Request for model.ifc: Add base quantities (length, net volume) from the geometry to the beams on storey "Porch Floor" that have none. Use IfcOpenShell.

First a look at what the model holds.

```python
import ifcopenshell
import ifcopenshell.util.element
import ifcopenshell.util.unit

model = ifcopenshell.open("model.ifc")
print(model.schema)
for unit_type in ("LENGTHUNIT", "AREAUNIT", "VOLUMEUNIT"):
    print(unit_type, ifcopenshell.util.unit.calculate_unit_scale(model, unit_type))
storey = next(s for s in model.by_type("IfcBuildingStorey") if s.Name == "Porch Floor")
beams = [e for e in ifcopenshell.util.element.get_decomposition(storey) if e.is_a("IfcBeam")]
for e in sorted(beams, key=lambda e: e.id()):
    print(e.id(), e.is_a(), e.Name, list(ifcopenshell.util.element.get_psets(e, qtos_only=True)), sep=" | ")
```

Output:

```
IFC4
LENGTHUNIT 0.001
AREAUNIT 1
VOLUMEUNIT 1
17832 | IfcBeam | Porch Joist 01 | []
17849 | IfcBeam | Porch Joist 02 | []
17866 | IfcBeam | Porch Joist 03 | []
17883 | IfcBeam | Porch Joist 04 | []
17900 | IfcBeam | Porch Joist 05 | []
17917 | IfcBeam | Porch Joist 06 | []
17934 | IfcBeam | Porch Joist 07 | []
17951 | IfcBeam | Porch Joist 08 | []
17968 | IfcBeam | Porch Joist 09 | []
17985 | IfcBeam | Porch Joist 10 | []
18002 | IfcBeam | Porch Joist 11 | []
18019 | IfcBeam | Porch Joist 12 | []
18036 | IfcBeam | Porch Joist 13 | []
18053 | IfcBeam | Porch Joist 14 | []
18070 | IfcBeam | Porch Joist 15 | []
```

```python
import ifcopenshell
import ifcopenshell.api.pset
import ifcopenshell.geom
import ifcopenshell.util.element
import ifcopenshell.util.shape
import ifcopenshell.util.unit

model = ifcopenshell.open("model.ifc")
unit_scale = ifcopenshell.util.unit.calculate_unit_scale(model)
volume_scale = ifcopenshell.util.unit.calculate_unit_scale(model, "VOLUMEUNIT")
settings = ifcopenshell.geom.settings()

storey = next(s for s in model.by_type("IfcBuildingStorey") if s.Name == "Porch Floor")
beams = [e for e in ifcopenshell.util.element.get_decomposition(storey) if e.is_a("IfcBeam")]

for e in sorted(beams, key=lambda e: e.id()):
    if ifcopenshell.util.element.get_psets(e, qtos_only=True, should_inherit=False):
        continue
    # Geometry comes back in metres, in the element's own axes.
    shape = ifcopenshell.geom.create_shape(settings, e)
    values = {
        "Length": ifcopenshell.util.shape.get_max_xyz(shape.geometry) / unit_scale,
        "NetVolume": ifcopenshell.util.shape.get_volume(shape.geometry) / volume_scale,
    }
    qto = ifcopenshell.api.pset.add_qto(model, product=e, name="Qto_BeamBaseQuantities")
    ifcopenshell.api.pset.edit_qto(model, qto=qto, properties=values)
    print(e.id(), {k: round(v, 3) for k, v in values.items()})

model.write("model_rev.ifc")
```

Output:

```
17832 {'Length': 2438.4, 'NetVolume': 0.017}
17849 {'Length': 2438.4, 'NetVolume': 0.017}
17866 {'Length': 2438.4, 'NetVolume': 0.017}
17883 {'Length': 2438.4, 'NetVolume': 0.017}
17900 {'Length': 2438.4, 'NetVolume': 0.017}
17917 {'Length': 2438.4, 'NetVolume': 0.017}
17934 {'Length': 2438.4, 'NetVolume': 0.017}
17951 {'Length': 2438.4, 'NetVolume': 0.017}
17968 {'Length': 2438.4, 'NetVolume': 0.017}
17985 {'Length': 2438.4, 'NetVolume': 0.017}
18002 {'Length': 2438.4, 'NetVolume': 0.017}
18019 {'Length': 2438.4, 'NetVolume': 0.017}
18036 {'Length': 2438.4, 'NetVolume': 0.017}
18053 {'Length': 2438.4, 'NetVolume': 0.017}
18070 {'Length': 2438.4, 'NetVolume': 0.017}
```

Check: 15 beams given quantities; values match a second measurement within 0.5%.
